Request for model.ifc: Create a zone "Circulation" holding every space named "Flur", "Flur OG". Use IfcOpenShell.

First a look at what the model holds.

```python
import ifcopenshell

model = ifcopenshell.open("model.ifc")
print(model.schema)
seen = {}
for space in model.by_type("IfcSpace"):
    seen[space.LongName] = seen.get(space.LongName, 0) + 1
for name, count in sorted(seen.items(), key=str):
    print(count, "x", name)
print("zones:", [z.Name for z in model.by_type("IfcZone")][:20])
```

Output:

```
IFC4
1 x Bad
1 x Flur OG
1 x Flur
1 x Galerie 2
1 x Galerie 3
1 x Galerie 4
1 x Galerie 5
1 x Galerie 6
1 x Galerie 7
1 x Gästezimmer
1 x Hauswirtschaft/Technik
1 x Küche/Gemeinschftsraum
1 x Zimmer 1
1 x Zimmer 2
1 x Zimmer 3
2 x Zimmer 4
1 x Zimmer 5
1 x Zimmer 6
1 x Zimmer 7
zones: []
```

```python
import ifcopenshell
import ifcopenshell.api.group
import ifcopenshell.api.root

model = ifcopenshell.open("model.ifc")

names = {"Flur", "Flur OG"}
spaces = [s for s in model.by_type("IfcSpace") if s.LongName in names]

zone = ifcopenshell.api.root.create_entity(model, ifc_class="IfcZone", name="Circulation")
ifcopenshell.api.group.assign_group(model, products=spaces, group=zone)
print(len(spaces), "spaces in", zone.Name)

model.write("model_v2.ifc")
```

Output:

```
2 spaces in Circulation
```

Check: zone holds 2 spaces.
